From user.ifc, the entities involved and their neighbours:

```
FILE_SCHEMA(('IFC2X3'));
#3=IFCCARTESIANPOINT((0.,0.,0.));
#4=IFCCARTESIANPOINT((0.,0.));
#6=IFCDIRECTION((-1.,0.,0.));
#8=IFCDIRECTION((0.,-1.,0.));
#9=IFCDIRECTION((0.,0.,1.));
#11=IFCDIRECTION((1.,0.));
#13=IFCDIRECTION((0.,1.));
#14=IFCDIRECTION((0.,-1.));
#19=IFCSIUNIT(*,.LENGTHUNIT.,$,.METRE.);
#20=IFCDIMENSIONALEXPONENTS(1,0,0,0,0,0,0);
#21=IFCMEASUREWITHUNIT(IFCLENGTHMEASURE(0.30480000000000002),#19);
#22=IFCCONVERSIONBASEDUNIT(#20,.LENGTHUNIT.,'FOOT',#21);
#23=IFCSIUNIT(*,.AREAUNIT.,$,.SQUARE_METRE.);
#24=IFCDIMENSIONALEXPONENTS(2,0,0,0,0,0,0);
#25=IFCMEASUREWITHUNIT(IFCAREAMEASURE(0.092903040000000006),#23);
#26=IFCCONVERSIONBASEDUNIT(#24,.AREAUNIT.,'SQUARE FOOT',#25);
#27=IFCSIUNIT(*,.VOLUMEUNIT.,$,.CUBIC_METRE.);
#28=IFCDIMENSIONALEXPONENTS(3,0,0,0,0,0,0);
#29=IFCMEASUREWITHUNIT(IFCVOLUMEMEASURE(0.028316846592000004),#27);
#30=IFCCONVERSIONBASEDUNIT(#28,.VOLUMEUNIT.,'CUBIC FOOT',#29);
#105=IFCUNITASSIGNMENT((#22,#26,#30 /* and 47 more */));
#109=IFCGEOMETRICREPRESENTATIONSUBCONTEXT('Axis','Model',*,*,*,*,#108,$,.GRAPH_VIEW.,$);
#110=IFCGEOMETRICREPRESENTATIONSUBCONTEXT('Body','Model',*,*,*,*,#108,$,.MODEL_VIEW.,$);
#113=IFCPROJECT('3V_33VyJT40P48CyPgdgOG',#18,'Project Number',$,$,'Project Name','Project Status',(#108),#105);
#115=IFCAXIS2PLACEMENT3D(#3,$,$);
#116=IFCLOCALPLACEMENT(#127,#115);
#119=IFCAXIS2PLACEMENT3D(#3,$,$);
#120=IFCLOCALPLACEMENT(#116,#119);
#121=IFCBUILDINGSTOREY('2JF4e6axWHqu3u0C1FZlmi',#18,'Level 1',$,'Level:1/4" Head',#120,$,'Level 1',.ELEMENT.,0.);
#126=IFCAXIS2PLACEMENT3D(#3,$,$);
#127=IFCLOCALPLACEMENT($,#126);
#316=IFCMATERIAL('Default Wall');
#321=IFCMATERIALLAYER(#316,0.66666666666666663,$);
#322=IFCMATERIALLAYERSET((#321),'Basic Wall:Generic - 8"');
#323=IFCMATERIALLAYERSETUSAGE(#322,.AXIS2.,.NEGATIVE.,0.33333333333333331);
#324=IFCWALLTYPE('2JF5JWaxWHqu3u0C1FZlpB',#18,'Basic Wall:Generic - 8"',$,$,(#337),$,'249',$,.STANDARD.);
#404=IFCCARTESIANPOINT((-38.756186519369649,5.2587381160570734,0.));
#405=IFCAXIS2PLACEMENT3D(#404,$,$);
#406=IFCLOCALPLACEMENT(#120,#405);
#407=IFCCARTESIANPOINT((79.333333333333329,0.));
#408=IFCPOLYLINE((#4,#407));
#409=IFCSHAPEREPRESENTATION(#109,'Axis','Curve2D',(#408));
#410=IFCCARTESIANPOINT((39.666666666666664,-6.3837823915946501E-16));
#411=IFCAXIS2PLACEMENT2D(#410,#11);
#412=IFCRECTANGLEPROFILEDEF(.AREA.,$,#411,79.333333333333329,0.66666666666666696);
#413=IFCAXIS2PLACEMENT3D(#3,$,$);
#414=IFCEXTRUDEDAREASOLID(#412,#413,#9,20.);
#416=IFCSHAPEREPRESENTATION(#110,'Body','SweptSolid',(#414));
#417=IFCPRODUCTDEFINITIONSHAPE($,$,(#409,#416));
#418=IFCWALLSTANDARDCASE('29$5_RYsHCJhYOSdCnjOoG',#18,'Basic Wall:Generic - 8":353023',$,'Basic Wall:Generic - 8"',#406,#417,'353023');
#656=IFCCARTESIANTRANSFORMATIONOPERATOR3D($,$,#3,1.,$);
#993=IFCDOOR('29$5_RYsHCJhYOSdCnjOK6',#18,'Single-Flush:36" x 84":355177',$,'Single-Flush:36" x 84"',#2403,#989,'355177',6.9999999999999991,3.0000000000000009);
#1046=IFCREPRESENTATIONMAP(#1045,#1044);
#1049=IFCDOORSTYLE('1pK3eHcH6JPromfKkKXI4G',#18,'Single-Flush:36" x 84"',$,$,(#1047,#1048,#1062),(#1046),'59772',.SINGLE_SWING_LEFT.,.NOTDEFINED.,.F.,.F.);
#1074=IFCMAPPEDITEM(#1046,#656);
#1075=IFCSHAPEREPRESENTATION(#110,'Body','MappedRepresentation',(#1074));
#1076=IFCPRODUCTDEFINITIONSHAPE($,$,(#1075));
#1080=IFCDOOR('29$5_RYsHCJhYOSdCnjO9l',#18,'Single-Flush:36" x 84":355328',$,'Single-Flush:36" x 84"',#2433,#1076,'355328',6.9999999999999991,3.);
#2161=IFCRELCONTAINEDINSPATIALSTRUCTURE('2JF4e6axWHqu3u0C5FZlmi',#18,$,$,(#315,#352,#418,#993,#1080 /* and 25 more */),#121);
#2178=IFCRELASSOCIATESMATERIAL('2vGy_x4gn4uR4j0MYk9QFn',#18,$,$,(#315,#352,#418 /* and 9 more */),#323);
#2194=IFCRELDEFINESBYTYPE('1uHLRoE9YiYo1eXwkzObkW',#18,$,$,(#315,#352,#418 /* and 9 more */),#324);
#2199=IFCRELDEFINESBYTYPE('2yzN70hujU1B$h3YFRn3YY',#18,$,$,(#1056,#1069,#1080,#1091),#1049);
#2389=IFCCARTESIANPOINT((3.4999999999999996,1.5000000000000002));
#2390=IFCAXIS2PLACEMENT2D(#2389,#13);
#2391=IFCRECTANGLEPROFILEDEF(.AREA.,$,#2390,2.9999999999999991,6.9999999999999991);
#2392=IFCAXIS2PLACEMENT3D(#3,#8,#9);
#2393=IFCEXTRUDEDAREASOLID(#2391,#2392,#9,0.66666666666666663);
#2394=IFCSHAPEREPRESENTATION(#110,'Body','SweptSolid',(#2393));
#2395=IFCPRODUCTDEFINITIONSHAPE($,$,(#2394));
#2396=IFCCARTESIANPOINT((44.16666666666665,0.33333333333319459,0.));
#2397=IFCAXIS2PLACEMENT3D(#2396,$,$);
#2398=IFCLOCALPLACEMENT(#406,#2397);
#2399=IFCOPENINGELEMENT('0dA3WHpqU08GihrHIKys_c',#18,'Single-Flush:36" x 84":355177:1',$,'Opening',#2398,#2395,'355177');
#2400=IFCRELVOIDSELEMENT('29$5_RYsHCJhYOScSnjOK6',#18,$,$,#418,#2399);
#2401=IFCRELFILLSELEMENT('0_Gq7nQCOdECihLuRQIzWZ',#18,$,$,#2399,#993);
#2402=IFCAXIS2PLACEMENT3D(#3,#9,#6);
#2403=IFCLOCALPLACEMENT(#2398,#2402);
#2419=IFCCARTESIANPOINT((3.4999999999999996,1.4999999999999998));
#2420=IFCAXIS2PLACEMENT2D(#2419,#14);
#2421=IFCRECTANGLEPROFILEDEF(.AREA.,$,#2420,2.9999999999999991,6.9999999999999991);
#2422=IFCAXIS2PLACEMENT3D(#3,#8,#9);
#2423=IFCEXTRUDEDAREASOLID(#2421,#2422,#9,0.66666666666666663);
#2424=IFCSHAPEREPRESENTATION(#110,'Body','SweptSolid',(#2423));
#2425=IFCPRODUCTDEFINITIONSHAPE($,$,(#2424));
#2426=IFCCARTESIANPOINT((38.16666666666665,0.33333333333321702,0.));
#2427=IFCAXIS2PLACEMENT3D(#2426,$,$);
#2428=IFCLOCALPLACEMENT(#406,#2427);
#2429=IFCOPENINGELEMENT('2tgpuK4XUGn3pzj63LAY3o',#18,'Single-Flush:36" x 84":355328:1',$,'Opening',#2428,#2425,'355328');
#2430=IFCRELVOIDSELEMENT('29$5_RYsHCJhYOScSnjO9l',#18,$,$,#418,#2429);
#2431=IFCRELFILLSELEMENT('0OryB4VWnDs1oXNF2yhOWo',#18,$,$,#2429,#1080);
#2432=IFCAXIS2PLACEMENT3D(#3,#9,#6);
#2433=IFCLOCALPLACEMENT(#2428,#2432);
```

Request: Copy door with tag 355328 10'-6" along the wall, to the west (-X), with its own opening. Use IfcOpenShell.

```python
import ifcopenshell
import ifcopenshell.api.feature
import ifcopenshell.api.geometry
import ifcopenshell.api.root
import ifcopenshell.geom
import ifcopenshell.util.element
import ifcopenshell.util.placement
import ifcopenshell.util.shape
import ifcopenshell.util.unit

model = ifcopenshell.open("user.ifc")
unit_scale = ifcopenshell.util.unit.calculate_unit_scale(model)
settings = ifcopenshell.geom.settings()


def volume(element):
    """Net volume in cubic metres, openings subtracted."""
    shape = ifcopenshell.geom.create_shape(settings, element)
    return ifcopenshell.util.shape.get_volume(shape.geometry)


def reuse_history(source, copy):
    """copy_class also copies each property set's owner history, people and application; keep the originals."""
    for rel in copy.IsDefinedBy:
        if rel.is_a("IfcRelDefinesByProperties") and (history := rel.RelatingPropertyDefinition.OwnerHistory):
            rel.RelatingPropertyDefinition.OwnerHistory = source.OwnerHistory
            ifcopenshell.util.element.remove_deep2(model, history)


door = model.by_guid("29$5_RYsHCJhYOSdCnjO9l")
opening = door.FillsVoids[0].RelatingOpeningElement
wall = opening.VoidsElements[0].RelatingBuildingElement
before = volume(wall)
shift = ifcopenshell.util.placement.get_local_placement(wall.ObjectPlacement)[:3, 0] * -126 * 0.0254 / unit_scale

# copy_class copies the void relationship, type, container and properties, but no geometry.
new_opening = ifcopenshell.api.root.copy_class(model, product=opening)
new_opening.Representation = ifcopenshell.util.element.copy_deep(
    model, opening.Representation, exclude=["IfcGeometricRepresentationContext", "IfcRepresentationMap"]
)
new_opening.Name = 'Single-Flush:36" x 84"'
new_opening.Tag = None
new_door = ifcopenshell.api.root.copy_class(model, product=door)
new_door.Representation = ifcopenshell.util.element.copy_deep(
    model, door.Representation, exclude=["IfcGeometricRepresentationContext", "IfcRepresentationMap"]
)
new_door.Name = 'Single-Flush:36" x 84"'
new_door.Tag = None
reuse_history(door, new_door)
fills = ifcopenshell.api.feature.add_filling(model, opening=new_opening, element=new_door)
fills.OwnerHistory = new_door.OwnerHistory  # required in IFC2X3

for old, new in ((opening, new_opening), (door, new_door)):
    matrix = ifcopenshell.util.placement.get_local_placement(old.ObjectPlacement)
    matrix[:3, 3] += shift
    ifcopenshell.api.geometry.edit_object_placement(model, product=new, matrix=matrix, is_si=False)

after = volume(wall)

print(f"wall volume {before:.3f} -> {after:.3f} m3")

model.write("user_rev.ifc")
```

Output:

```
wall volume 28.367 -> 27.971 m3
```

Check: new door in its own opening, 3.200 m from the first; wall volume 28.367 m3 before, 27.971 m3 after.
